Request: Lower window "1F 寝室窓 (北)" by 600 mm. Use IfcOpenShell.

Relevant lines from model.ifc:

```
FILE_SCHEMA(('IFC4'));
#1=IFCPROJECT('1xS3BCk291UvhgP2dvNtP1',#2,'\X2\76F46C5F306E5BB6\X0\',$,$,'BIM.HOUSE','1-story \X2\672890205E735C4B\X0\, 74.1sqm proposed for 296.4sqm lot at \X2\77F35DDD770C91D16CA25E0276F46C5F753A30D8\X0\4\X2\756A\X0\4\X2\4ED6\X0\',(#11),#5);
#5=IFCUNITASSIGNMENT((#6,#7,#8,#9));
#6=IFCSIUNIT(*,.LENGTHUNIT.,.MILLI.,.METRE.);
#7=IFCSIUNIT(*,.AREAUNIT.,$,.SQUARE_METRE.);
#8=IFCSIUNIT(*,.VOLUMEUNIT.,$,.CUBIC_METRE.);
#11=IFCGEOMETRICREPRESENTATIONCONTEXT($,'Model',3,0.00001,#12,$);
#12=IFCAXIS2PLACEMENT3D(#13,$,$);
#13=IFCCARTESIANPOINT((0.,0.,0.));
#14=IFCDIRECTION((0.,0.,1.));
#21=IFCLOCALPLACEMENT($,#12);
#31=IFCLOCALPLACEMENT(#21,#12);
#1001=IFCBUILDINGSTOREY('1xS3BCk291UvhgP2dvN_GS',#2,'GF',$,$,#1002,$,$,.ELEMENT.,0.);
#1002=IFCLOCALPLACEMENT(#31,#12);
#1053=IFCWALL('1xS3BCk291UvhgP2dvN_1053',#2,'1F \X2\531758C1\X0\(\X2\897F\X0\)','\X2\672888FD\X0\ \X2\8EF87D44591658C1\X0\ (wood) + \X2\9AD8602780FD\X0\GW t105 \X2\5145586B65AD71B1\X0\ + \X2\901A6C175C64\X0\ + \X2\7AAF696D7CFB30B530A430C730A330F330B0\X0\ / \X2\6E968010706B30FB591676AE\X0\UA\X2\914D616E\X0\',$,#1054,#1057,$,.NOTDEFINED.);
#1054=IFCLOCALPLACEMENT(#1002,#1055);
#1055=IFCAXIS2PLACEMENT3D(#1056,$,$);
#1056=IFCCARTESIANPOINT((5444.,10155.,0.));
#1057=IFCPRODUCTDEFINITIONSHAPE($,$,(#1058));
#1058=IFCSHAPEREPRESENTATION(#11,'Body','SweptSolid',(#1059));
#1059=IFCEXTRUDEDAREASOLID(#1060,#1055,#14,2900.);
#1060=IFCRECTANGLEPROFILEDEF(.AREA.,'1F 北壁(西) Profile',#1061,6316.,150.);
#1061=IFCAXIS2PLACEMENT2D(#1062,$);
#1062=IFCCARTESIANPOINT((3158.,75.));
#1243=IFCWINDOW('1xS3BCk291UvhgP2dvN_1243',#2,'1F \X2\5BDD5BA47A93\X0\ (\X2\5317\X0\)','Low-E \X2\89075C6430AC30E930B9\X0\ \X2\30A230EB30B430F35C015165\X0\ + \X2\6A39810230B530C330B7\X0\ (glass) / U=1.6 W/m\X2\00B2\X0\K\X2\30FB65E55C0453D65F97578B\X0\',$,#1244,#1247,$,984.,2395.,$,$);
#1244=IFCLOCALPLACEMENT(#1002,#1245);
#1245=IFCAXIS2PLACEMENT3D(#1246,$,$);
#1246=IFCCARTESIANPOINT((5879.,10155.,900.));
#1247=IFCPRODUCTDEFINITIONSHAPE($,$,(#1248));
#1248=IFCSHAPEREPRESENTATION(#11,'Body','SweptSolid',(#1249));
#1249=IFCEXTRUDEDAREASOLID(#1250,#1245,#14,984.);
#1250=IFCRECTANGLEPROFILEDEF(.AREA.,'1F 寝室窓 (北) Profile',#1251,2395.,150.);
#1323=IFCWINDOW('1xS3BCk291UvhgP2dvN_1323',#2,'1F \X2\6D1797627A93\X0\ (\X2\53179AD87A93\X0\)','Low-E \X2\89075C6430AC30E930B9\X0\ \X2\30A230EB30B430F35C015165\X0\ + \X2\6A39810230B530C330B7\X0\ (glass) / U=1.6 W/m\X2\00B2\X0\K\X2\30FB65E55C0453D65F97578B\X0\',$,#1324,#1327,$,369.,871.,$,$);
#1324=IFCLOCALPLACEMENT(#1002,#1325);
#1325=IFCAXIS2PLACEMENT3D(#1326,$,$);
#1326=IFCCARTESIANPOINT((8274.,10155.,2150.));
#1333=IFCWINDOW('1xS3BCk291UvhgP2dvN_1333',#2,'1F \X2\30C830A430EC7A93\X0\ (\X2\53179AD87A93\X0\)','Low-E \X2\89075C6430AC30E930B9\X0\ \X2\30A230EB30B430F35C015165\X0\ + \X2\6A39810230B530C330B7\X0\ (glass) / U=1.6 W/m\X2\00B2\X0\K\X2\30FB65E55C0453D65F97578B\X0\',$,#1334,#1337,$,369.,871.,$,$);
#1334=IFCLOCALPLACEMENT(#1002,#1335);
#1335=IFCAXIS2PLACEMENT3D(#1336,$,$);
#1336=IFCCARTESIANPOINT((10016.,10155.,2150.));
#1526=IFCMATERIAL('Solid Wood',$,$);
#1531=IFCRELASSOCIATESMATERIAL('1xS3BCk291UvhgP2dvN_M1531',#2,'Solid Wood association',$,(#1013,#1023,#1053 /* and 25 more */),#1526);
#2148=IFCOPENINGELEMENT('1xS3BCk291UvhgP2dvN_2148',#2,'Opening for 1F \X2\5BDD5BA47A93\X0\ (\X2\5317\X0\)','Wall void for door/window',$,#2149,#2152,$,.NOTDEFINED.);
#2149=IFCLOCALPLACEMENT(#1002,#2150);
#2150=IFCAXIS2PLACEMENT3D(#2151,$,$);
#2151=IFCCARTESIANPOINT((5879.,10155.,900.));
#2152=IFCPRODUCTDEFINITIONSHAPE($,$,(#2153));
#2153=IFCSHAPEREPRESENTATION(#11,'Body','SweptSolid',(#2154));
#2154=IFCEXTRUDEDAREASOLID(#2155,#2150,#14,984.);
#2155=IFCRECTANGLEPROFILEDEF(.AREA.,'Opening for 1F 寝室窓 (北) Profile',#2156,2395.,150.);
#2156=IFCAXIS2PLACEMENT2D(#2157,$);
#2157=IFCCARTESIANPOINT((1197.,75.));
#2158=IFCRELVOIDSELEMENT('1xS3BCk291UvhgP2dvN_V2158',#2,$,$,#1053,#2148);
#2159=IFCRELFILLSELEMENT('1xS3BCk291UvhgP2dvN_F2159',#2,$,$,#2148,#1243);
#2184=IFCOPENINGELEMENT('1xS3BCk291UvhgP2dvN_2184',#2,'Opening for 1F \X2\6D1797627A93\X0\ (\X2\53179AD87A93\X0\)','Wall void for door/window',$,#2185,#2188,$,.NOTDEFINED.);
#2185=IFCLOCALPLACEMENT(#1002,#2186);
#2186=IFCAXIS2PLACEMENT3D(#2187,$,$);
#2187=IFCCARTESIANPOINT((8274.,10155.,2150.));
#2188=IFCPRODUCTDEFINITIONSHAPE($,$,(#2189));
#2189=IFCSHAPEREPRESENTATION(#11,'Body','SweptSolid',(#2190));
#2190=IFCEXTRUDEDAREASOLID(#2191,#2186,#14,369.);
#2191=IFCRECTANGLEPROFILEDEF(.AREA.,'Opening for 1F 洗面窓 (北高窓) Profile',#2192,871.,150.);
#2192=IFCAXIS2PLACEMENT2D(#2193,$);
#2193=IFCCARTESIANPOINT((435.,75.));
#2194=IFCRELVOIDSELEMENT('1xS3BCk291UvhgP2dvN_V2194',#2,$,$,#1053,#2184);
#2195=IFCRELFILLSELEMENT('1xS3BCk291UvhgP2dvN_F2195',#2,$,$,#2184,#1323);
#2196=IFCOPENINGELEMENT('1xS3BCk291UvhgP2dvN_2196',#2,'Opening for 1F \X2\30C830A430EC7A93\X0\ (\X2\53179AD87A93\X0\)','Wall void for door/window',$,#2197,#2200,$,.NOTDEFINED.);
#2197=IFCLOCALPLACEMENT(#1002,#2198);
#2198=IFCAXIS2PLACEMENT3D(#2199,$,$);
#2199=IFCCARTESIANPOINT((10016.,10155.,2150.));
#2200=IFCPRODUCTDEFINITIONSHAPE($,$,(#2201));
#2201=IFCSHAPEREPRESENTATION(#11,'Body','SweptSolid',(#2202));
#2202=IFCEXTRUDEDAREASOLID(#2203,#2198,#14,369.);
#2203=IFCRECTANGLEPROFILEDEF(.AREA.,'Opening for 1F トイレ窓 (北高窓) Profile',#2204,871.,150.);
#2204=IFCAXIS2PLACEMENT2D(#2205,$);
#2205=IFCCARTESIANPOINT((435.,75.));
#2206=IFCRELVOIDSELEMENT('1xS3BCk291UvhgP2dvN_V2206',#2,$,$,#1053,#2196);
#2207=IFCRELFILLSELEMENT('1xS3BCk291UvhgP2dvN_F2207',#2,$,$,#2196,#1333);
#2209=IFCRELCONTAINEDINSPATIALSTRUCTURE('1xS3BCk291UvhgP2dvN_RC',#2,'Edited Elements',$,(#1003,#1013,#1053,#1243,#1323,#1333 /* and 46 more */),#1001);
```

```python
import numpy as np
import ifcopenshell
import ifcopenshell.api.geometry
import ifcopenshell.util.placement
import ifcopenshell.util.unit

model = ifcopenshell.open("model.ifc")
unit_scale = ifcopenshell.util.unit.calculate_unit_scale(model)

window = model.by_id(1243)
opening = window.FillsVoids[0].RelatingOpeningElement
dz = -600.0

shift = np.array([0.0, 0.0, dz])
# The window is not placed relative to its opening, so move both.
for product in (opening, window):
    matrix = ifcopenshell.util.placement.get_local_placement(product.ObjectPlacement)
    matrix[:3, 3] += shift
    ifcopenshell.api.geometry.edit_object_placement(model, product=product, matrix=matrix, is_si=False)

print(f"moved by {dz * unit_scale:+.3f} m")

model.write("model_updated.ifc")
```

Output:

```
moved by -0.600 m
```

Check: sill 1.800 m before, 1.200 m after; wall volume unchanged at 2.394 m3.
